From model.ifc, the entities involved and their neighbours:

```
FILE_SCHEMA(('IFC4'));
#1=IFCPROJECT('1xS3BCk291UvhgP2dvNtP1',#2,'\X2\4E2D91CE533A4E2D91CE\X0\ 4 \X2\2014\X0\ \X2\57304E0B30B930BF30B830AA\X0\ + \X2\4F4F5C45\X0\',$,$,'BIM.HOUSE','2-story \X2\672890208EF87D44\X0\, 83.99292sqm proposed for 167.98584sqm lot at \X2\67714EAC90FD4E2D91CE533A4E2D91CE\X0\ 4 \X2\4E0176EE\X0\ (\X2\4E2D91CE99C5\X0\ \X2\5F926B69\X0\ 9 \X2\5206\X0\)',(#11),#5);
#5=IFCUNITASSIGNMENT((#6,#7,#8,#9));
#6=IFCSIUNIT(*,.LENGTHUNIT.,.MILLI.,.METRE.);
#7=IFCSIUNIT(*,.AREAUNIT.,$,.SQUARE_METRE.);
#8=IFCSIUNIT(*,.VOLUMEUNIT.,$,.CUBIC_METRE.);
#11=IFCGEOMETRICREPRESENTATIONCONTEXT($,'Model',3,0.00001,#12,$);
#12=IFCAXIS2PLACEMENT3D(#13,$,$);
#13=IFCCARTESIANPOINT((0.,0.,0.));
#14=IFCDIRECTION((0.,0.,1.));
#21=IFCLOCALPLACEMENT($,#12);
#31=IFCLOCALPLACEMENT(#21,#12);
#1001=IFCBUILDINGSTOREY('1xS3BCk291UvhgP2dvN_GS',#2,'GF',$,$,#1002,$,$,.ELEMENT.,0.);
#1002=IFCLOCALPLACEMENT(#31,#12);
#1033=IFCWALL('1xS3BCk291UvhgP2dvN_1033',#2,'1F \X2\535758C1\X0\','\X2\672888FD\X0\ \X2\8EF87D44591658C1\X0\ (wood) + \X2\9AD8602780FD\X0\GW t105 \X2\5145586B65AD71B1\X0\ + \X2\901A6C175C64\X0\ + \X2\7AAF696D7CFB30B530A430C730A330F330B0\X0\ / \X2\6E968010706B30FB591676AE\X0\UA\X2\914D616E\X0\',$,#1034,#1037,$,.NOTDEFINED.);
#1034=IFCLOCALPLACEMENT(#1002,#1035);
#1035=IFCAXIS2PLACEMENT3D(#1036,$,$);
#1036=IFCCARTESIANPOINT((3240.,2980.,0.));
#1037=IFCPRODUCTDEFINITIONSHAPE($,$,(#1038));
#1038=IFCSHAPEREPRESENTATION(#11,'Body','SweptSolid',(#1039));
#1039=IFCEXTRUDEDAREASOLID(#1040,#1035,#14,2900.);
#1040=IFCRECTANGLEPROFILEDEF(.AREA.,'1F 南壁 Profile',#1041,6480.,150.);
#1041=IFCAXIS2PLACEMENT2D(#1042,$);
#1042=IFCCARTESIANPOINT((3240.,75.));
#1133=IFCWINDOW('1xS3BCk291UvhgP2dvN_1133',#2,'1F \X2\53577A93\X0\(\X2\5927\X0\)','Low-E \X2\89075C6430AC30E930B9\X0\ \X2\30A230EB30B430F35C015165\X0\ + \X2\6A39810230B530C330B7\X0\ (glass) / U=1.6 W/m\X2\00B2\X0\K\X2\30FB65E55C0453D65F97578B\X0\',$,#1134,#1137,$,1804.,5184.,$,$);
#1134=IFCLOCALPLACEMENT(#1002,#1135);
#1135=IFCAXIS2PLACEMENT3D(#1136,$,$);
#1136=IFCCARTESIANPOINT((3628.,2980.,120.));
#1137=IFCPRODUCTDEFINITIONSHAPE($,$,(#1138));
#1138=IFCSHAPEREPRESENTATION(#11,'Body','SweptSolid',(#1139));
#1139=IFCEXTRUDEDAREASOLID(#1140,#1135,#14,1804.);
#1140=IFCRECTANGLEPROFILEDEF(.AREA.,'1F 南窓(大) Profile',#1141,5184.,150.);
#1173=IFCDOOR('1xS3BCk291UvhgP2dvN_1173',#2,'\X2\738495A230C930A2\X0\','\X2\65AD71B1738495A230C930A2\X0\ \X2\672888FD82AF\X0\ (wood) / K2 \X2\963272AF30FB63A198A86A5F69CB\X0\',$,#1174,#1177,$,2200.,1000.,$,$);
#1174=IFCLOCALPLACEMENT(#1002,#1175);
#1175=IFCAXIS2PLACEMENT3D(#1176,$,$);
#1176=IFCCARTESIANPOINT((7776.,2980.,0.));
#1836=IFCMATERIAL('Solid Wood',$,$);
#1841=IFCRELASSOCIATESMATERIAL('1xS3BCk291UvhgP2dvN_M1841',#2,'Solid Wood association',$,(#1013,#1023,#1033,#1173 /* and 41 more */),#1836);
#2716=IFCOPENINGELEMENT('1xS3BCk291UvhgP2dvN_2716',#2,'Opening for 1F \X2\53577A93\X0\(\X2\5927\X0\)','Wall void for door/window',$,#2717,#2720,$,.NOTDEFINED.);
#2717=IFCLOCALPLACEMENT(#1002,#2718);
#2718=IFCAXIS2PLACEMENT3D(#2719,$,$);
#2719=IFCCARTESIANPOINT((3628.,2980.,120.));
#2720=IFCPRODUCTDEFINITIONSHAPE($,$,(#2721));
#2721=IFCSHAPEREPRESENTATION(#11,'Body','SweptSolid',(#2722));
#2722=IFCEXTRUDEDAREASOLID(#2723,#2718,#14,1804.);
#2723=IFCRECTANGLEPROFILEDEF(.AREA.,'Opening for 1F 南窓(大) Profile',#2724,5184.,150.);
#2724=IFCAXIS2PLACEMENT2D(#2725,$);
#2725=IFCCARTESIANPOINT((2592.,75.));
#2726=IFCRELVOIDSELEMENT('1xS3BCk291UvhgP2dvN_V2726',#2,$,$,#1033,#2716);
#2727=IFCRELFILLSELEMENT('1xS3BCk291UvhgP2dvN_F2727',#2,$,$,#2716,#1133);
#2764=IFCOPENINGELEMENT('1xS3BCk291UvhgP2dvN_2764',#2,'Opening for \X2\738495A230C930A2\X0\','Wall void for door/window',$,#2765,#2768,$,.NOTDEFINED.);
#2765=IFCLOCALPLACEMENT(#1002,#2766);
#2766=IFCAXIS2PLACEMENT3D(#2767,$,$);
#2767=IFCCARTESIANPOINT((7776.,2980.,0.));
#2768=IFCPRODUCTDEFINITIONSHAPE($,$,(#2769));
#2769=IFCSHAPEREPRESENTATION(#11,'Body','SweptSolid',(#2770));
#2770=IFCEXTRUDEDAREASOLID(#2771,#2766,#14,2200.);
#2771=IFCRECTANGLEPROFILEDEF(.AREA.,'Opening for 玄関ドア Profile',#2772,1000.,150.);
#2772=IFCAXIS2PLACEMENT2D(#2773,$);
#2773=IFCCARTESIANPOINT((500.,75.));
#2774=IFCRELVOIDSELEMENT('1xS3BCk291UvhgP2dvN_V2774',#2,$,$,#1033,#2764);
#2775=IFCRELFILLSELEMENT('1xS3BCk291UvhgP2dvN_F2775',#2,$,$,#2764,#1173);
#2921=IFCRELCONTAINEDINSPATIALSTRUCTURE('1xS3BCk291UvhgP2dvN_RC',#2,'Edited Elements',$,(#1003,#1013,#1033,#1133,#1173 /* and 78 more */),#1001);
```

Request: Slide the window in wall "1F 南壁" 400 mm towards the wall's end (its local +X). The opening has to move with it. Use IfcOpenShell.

```python
import ifcopenshell
import ifcopenshell.api.geometry
import ifcopenshell.util.placement
import ifcopenshell.util.unit

model = ifcopenshell.open("model.ifc")
unit_scale = ifcopenshell.util.unit.calculate_unit_scale(model)

window = model.by_guid("1xS3BCk291UvhgP2dvN_1133")
opening = window.FillsVoids[0].RelatingOpeningElement
wall = opening.VoidsElements[0].RelatingBuildingElement

wall_matrix = ifcopenshell.util.placement.get_local_placement(wall.ObjectPlacement)
shift = wall_matrix[:3, 0] * 0.4 / unit_scale
before = ifcopenshell.util.placement.get_local_placement(window.ObjectPlacement)[:3, 3].copy()

# The window is not placed relative to its opening, so move both.
for product in (opening, window):
    matrix = ifcopenshell.util.placement.get_local_placement(product.ObjectPlacement)
    matrix[:3, 3] += shift
    ifcopenshell.api.geometry.edit_object_placement(model, product=product, matrix=matrix, is_si=False)

after = ifcopenshell.util.placement.get_local_placement(window.ObjectPlacement)[:3, 3]
print("window moved by", (after - before).round(3) + 0.0)

model.write("model_v2.ifc")
```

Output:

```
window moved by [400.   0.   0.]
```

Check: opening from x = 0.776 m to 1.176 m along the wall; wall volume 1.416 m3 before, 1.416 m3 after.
